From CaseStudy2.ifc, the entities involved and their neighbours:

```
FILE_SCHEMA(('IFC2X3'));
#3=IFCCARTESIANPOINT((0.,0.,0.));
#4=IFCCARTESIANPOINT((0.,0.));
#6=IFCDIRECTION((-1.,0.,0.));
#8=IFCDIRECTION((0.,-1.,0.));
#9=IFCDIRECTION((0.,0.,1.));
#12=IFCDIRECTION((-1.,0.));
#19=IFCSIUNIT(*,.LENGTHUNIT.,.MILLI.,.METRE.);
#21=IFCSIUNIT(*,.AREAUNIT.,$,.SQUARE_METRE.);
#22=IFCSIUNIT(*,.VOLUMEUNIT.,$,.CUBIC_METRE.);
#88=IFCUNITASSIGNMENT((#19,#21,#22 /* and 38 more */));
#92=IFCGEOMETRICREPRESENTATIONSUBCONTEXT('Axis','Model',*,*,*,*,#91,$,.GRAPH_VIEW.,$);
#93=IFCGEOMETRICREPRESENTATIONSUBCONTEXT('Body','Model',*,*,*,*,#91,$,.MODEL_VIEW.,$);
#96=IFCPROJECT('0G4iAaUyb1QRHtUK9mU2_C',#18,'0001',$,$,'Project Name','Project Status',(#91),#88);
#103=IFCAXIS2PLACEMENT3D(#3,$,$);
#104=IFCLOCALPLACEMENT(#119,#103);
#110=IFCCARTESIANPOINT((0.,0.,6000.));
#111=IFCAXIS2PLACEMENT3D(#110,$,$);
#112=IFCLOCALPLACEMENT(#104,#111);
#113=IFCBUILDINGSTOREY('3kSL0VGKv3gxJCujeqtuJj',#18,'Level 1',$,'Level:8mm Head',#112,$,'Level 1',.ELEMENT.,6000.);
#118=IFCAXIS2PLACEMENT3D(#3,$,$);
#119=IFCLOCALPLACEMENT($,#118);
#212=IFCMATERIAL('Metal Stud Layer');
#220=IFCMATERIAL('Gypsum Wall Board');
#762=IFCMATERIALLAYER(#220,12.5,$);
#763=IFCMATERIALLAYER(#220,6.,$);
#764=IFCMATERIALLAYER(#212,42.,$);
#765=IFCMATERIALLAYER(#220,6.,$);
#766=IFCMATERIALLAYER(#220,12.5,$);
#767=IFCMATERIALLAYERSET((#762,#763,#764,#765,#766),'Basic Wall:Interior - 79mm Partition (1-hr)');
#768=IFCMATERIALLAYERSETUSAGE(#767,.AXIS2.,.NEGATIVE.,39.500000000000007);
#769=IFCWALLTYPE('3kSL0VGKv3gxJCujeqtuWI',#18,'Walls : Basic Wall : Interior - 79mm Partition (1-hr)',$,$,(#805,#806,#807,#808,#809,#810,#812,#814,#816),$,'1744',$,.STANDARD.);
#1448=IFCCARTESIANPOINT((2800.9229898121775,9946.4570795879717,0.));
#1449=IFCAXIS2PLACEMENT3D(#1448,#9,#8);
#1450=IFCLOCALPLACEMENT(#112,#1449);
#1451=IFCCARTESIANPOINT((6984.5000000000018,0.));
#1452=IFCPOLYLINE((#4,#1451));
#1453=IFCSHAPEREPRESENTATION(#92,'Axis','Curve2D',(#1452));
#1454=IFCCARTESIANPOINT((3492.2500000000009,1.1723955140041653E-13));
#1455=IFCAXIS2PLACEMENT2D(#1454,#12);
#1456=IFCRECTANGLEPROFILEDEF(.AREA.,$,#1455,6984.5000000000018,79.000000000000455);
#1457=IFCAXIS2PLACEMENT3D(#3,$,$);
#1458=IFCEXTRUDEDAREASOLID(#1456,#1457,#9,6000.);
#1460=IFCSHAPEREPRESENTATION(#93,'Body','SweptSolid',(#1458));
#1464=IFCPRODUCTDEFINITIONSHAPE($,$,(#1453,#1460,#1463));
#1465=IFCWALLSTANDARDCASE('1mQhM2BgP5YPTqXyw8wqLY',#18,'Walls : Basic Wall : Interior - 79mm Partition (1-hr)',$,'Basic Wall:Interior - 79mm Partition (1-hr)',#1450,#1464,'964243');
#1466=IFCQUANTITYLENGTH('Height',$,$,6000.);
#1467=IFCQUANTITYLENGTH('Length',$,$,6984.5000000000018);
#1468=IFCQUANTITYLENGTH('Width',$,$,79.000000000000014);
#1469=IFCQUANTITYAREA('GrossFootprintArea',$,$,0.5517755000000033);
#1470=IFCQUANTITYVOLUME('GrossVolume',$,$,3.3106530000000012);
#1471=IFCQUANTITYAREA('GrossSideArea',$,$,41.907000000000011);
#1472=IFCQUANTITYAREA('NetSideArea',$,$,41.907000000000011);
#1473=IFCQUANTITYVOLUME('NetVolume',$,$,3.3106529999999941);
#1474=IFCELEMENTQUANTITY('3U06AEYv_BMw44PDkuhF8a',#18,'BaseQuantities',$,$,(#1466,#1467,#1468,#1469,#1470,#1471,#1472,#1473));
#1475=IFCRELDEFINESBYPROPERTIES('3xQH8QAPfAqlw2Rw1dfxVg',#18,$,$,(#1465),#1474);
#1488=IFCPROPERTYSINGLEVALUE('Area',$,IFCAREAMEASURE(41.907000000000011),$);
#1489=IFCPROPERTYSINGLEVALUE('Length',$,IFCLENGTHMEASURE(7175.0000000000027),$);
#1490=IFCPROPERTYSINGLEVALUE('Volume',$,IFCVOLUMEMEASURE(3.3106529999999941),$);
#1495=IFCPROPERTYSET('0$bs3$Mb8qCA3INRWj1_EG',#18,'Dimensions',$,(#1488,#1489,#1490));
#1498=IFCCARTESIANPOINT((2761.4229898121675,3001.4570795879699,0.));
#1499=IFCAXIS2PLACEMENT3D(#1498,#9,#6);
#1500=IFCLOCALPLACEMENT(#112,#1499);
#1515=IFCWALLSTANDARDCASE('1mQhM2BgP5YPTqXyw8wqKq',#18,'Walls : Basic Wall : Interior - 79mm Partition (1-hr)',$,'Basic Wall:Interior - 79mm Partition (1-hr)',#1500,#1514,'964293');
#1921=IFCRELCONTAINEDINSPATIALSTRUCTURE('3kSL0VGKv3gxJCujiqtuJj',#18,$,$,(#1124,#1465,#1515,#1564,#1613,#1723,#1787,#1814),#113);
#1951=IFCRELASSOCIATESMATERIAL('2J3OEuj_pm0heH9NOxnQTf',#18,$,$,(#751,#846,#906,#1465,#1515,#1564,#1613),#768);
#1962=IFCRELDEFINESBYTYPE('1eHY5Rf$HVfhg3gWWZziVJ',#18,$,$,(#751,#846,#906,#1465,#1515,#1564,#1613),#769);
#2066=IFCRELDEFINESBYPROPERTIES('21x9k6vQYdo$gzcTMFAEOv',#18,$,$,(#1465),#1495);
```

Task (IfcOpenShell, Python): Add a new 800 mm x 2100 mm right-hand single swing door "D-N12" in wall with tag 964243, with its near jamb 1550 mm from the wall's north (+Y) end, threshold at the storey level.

```python
import numpy as np
import ifcopenshell
import ifcopenshell.api.feature
import ifcopenshell.api.geometry
import ifcopenshell.api.pset
import ifcopenshell.api.root
import ifcopenshell.api.spatial
import ifcopenshell.api.type
import ifcopenshell.geom
import ifcopenshell.util.element
import ifcopenshell.util.placement
import ifcopenshell.util.representation
import ifcopenshell.util.shape
import ifcopenshell.util.unit

model = ifcopenshell.open("CaseStudy2.ifc")
unit_scale = ifcopenshell.util.unit.calculate_unit_scale(model)
area_scale = ifcopenshell.util.unit.calculate_unit_scale(model, "AREAUNIT")
volume_scale = ifcopenshell.util.unit.calculate_unit_scale(model, "VOLUMEUNIT")
settings = ifcopenshell.geom.settings()


def volume(element):
    """Net volume in cubic metres, openings subtracted."""
    shape = ifcopenshell.geom.create_shape(settings, element)
    return ifcopenshell.util.shape.get_volume(shape.geometry)


wall = model.by_guid("1mQhM2BgP5YPTqXyw8wqLY")
storey = ifcopenshell.util.element.get_container(wall, ifc_class="IfcBuildingStorey")
context = ifcopenshell.util.representation.get_context(model, "Model", "Body", "MODEL_VIEW")
before = volume(wall)

width, height, from_end, sill = 0.8, 2.1, 1.55, 0.0  # metres

# The wall runs along its own X axis, and the end named is its -X end.
wall_shape = ifcopenshell.geom.create_shape(settings, wall)
x, y, z = ifcopenshell.util.shape.get_vertices(wall_shape.geometry).T
start = x.min() + from_end
face, thickness = float(y.min()), float(y.max() - y.min())
wall_matrix = ifcopenshell.util.placement.get_local_placement(wall.ObjectPlacement)
level = ifcopenshell.util.placement.get_local_placement(storey.ObjectPlacement)[2, 3]


def in_wall(x, y):
    """Placement at x, y metres in the wall's axes, at sill height."""
    matrix = wall_matrix.copy()
    matrix[:, 3] = wall_matrix @ np.array([x / unit_scale, y / unit_scale, 0.0, 1.0])
    matrix[2, 3] = level + sill / unit_scale
    return matrix


# Opening: a box that overshoots both wall faces by 50 mm.
opening = ifcopenshell.api.root.create_entity(model, ifc_class="IfcOpeningElement")
box = ifcopenshell.api.geometry.add_wall_representation(
    model, context=context, length=width, height=height, thickness=thickness + 0.1
)
ifcopenshell.api.geometry.assign_representation(model, product=opening, representation=box)
ifcopenshell.api.geometry.edit_object_placement(model, product=opening, matrix=in_wall(start, face - 0.05), is_si=False)
ifcopenshell.api.feature.add_feature(model, feature=opening, element=wall)

door = ifcopenshell.api.root.create_entity(model, ifc_class="IfcDoor", name="D-N12")
door.OverallWidth, door.OverallHeight = width / unit_scale, height / unit_scale
body = ifcopenshell.api.geometry.add_door_representation(
    model,
    context=context,
    overall_width=door.OverallWidth,
    overall_height=door.OverallHeight,
    operation_type="SINGLE_SWING_RIGHT",
    lining_properties={"LiningDepth": thickness / unit_scale, "ThresholdDepth": thickness / unit_scale},
)
ifcopenshell.api.geometry.assign_representation(model, product=door, representation=body)
ifcopenshell.api.spatial.assign_container(model, products=[door], relating_structure=storey)
fills = ifcopenshell.api.feature.add_filling(model, opening=opening, element=door)
fills.OwnerHistory = door.OwnerHistory  # required in IFC2X3

# IFC2X3 keeps the operation on the door style.
style = ifcopenshell.api.root.create_entity(model, ifc_class="IfcDoorStyle", name="D-N12")
style.OperationType, style.ConstructionType = "SINGLE_SWING_RIGHT", "NOTDEFINED"
style.ParameterTakesPrecedence = style.Sizeable = False
ifcopenshell.api.type.assign_type(model, related_objects=[door], relating_type=style)

# The lining spans the wall, so the door starts at the wall face.
ifcopenshell.api.geometry.edit_object_placement(model, product=door, matrix=in_wall(start, face), is_si=False)

after = volume(wall)

# Update the wall's stored quantities.
qto = model.by_id(ifcopenshell.util.element.get_pset(wall, "BaseQuantities", should_inherit=False)["id"])
ifcopenshell.api.pset.edit_qto(model, qto=qto, properties={
    "NetSideArea": after / thickness / area_scale,
    "NetVolume": after / volume_scale,
})
pset = model.by_id(ifcopenshell.util.element.get_pset(wall, "Dimensions", should_inherit=False)["id"])
ifcopenshell.api.pset.edit_pset(model, pset=pset, properties={
    "Area": model.create_entity("IfcAreaMeasure", after / thickness / area_scale),
    "Volume": model.create_entity("IfcVolumeMeasure", after / volume_scale),
})

print(f"wall volume {before:.3f} -> {after:.3f} m3")

model.write("CaseStudy2_edited.ifc")
```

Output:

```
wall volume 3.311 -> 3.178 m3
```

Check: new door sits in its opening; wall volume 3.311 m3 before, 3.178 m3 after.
